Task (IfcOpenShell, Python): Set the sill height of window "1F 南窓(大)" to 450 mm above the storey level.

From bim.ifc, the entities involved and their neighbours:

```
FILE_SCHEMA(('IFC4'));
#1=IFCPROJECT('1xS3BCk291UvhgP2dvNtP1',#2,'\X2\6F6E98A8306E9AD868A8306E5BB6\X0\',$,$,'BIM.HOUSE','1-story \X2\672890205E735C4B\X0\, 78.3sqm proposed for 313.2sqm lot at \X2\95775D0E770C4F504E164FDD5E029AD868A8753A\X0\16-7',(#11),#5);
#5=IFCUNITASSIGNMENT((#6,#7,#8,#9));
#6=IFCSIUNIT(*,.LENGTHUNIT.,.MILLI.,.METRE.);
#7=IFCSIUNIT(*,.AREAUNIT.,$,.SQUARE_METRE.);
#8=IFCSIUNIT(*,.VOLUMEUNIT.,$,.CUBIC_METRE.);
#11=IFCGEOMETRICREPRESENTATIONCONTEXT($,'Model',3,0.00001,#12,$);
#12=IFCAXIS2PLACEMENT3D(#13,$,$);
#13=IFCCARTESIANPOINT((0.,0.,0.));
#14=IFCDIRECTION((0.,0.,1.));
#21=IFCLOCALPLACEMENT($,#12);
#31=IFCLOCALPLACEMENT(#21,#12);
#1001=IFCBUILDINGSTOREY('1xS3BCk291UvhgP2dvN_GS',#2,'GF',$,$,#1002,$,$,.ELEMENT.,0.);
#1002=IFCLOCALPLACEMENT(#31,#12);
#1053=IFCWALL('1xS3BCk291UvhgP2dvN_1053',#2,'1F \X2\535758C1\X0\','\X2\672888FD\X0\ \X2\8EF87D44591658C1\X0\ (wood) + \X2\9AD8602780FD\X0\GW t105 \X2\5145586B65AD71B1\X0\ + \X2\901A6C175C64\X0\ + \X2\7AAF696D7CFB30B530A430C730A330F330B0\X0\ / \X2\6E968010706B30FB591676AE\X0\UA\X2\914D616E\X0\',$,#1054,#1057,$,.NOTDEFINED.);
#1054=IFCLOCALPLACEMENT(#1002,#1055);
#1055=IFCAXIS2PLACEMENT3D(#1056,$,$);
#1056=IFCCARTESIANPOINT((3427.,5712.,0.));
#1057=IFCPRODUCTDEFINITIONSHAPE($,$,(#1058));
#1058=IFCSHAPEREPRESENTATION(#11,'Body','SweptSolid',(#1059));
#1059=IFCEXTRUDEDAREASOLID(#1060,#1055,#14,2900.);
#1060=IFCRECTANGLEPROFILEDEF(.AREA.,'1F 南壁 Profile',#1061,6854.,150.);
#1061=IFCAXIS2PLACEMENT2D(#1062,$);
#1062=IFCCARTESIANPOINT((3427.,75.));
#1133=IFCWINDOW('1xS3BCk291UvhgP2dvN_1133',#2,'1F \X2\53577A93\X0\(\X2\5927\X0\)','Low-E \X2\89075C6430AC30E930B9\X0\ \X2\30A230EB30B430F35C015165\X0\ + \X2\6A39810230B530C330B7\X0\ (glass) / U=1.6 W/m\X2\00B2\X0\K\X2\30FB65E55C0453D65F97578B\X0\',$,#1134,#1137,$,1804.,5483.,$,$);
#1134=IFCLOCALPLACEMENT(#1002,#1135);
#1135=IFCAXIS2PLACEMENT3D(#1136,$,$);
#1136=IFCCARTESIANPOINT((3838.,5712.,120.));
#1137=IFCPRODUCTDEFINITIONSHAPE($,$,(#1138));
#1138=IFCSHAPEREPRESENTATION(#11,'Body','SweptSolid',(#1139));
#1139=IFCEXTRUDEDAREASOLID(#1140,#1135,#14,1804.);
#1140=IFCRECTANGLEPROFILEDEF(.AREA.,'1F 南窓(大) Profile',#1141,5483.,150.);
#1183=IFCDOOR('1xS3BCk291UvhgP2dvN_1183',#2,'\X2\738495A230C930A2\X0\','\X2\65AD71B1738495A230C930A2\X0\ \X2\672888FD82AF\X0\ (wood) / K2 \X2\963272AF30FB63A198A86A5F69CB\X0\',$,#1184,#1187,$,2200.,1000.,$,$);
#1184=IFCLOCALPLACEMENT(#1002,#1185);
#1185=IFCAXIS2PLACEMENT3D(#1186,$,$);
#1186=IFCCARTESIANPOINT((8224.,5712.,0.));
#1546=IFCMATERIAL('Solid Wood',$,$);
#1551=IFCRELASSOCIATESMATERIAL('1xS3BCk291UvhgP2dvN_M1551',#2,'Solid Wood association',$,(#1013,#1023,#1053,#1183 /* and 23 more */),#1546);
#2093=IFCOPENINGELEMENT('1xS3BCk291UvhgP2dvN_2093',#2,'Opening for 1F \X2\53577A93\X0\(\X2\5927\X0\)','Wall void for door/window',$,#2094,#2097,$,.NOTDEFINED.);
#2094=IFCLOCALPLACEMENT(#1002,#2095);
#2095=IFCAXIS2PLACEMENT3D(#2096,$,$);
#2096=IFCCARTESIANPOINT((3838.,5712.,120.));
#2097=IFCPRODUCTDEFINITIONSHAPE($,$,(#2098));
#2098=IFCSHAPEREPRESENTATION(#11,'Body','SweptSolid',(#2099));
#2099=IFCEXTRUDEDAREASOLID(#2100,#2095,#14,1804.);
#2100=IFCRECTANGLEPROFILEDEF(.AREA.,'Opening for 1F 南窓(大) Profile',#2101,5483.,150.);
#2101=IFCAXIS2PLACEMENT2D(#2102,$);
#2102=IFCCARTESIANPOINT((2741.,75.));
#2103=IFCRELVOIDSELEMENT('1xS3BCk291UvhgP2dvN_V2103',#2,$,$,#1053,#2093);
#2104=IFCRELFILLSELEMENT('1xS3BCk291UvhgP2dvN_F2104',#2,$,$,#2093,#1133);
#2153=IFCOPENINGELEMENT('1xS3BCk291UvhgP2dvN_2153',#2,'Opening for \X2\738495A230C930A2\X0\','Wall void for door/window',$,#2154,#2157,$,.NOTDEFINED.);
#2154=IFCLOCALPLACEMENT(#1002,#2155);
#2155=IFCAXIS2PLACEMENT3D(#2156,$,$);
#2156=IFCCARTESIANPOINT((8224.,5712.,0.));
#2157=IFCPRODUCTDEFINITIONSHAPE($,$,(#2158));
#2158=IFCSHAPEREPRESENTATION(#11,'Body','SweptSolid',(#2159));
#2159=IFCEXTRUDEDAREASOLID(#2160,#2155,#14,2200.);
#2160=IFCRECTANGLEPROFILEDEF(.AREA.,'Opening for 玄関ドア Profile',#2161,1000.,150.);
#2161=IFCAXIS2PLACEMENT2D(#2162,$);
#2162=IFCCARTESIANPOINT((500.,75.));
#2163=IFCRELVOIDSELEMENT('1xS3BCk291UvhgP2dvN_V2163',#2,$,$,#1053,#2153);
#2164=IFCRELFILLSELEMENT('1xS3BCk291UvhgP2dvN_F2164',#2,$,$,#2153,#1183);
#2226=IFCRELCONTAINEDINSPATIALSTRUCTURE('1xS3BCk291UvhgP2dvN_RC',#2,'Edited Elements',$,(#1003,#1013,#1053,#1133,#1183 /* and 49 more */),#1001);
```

```python
import numpy as np
import ifcopenshell
import ifcopenshell.api.geometry
import ifcopenshell.geom
import ifcopenshell.util.element
import ifcopenshell.util.placement
import ifcopenshell.util.shape
import ifcopenshell.util.unit

model = ifcopenshell.open("bim.ifc")
unit_scale = ifcopenshell.util.unit.calculate_unit_scale(model)

window = model.by_guid("1xS3BCk291UvhgP2dvN_1133")
opening = window.FillsVoids[0].RelatingOpeningElement
storey = ifcopenshell.util.element.get_container(window, ifc_class="IfcBuildingStorey")
level = ifcopenshell.util.placement.get_local_placement(storey.ObjectPlacement)[2, 3]

# The opening's origin need not be at the sill, so measure its lowest point.
shape = ifcopenshell.geom.create_shape(ifcopenshell.geom.settings(), opening)
bottom = ifcopenshell.util.shape.get_shape_bottom_elevation(shape, shape.geometry) / unit_scale
dz = level + 0.45 / unit_scale - bottom

shift = np.array([0.0, 0.0, dz])
# The window is not placed relative to its opening, so move both.
for product in (opening, window):
    matrix = ifcopenshell.util.placement.get_local_placement(product.ObjectPlacement)
    matrix[:3, 3] += shift
    ifcopenshell.api.geometry.edit_object_placement(model, product=product, matrix=matrix, is_si=False)

print(f"moved by {dz * unit_scale:+.3f} m")

model.write("bim-out.ifc")
```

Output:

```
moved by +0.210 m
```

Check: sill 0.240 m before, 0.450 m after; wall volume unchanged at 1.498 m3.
